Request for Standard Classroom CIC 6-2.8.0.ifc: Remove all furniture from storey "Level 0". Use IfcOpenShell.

First a look at what the model holds.

```python
import ifcopenshell
import ifcopenshell.util.element

model = ifcopenshell.open("Standard Classroom CIC 6-2.8.0.ifc")
print(model.schema)
storey = next(s for s in model.by_type("IfcBuildingStorey") if s.Name == "Level 0")
furniture = [e for e in ifcopenshell.util.element.get_decomposition(storey) if e.is_a("IfcFurnishingElement")]
seen = {}
for e in furniture:
    element_type = ifcopenshell.util.element.get_type(e)
    name = element_type.Name if element_type not in (None, e) else None
    seen[name] = seen.get(name, 0) + 1
for name, count in sorted(seen.items(), key=str):
    print(count, "x", name)
```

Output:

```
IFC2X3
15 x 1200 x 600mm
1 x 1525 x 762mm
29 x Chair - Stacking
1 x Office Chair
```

```python
import ifcopenshell
import ifcopenshell.api.root
import ifcopenshell.util.element

model = ifcopenshell.open("Standard Classroom CIC 6-2.8.0.ifc")

storey = next(s for s in model.by_type("IfcBuildingStorey") if s.Name == "Level 0")
furniture = [e for e in ifcopenshell.util.element.get_decomposition(storey) if e.is_a("IfcFurnishingElement")]

for e in furniture:
    ifcopenshell.api.root.remove_product(model, product=e)
print(len(furniture), "removed")

model.write("Standard Classroom CIC 6-2.8.0-out.ifc")
```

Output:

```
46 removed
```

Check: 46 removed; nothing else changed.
